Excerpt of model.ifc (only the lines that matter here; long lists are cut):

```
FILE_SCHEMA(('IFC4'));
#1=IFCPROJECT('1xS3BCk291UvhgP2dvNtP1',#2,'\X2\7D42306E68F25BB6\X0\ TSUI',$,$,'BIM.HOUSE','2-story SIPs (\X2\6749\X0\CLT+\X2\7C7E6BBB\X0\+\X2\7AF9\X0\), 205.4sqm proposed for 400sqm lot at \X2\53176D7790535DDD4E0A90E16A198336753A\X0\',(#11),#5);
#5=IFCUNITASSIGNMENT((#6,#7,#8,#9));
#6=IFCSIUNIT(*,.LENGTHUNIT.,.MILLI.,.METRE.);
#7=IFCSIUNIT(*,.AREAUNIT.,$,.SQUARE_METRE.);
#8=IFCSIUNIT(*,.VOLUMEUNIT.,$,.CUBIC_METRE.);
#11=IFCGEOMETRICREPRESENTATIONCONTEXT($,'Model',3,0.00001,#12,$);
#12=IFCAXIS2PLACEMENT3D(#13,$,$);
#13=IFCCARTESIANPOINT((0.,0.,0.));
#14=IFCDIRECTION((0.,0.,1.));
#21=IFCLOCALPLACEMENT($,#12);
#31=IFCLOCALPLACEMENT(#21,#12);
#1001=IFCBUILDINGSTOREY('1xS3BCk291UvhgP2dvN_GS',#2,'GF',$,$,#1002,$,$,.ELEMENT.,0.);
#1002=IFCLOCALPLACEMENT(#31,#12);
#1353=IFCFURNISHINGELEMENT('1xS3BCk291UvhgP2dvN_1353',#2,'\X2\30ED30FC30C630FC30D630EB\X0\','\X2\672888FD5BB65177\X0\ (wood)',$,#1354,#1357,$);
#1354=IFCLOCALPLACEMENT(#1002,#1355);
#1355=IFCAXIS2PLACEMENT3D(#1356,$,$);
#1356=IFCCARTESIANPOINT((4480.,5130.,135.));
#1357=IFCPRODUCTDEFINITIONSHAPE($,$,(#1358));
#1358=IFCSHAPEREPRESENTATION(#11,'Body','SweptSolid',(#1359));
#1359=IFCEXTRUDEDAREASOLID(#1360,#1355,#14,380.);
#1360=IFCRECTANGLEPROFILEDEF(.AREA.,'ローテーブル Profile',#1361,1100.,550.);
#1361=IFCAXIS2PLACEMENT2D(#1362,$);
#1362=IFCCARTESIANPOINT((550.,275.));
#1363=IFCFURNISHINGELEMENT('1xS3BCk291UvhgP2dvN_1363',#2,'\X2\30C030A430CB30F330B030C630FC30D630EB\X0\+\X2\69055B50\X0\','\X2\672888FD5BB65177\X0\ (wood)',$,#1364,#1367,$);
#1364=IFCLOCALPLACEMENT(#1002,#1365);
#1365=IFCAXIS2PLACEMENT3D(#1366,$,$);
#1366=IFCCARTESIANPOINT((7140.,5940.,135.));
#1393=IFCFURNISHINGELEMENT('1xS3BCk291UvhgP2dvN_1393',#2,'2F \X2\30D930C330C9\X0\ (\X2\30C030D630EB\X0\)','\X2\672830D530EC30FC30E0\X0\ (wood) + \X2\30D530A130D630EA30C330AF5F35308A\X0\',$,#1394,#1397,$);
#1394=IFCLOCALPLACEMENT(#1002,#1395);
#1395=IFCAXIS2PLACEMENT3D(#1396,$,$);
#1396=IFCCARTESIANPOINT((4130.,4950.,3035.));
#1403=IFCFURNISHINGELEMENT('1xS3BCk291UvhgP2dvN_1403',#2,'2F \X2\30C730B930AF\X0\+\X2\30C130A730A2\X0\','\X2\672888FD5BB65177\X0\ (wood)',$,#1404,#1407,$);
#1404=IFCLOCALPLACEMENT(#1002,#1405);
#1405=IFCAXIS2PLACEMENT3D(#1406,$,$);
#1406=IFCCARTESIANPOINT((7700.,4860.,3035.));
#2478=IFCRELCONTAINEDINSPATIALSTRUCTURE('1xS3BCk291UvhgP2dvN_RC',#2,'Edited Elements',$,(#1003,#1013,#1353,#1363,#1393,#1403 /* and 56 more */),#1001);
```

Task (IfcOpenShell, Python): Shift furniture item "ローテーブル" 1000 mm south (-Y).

```python
import ifcopenshell
import ifcopenshell.api.geometry
import ifcopenshell.util.placement

model = ifcopenshell.open("model.ifc")

item = model.by_id(1353)
matrix = ifcopenshell.util.placement.get_local_placement(item.ObjectPlacement)
matrix[1, 3] -= 1000.0
ifcopenshell.api.geometry.edit_object_placement(model, product=item, matrix=matrix, is_si=False)

print(ifcopenshell.util.placement.get_local_placement(item.ObjectPlacement).round(3) + 0.0)

model.write("model_v2.ifc")
```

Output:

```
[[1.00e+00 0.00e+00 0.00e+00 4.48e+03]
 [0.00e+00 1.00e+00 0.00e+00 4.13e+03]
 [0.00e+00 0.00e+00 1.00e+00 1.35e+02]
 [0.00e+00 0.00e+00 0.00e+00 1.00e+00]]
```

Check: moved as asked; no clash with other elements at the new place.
